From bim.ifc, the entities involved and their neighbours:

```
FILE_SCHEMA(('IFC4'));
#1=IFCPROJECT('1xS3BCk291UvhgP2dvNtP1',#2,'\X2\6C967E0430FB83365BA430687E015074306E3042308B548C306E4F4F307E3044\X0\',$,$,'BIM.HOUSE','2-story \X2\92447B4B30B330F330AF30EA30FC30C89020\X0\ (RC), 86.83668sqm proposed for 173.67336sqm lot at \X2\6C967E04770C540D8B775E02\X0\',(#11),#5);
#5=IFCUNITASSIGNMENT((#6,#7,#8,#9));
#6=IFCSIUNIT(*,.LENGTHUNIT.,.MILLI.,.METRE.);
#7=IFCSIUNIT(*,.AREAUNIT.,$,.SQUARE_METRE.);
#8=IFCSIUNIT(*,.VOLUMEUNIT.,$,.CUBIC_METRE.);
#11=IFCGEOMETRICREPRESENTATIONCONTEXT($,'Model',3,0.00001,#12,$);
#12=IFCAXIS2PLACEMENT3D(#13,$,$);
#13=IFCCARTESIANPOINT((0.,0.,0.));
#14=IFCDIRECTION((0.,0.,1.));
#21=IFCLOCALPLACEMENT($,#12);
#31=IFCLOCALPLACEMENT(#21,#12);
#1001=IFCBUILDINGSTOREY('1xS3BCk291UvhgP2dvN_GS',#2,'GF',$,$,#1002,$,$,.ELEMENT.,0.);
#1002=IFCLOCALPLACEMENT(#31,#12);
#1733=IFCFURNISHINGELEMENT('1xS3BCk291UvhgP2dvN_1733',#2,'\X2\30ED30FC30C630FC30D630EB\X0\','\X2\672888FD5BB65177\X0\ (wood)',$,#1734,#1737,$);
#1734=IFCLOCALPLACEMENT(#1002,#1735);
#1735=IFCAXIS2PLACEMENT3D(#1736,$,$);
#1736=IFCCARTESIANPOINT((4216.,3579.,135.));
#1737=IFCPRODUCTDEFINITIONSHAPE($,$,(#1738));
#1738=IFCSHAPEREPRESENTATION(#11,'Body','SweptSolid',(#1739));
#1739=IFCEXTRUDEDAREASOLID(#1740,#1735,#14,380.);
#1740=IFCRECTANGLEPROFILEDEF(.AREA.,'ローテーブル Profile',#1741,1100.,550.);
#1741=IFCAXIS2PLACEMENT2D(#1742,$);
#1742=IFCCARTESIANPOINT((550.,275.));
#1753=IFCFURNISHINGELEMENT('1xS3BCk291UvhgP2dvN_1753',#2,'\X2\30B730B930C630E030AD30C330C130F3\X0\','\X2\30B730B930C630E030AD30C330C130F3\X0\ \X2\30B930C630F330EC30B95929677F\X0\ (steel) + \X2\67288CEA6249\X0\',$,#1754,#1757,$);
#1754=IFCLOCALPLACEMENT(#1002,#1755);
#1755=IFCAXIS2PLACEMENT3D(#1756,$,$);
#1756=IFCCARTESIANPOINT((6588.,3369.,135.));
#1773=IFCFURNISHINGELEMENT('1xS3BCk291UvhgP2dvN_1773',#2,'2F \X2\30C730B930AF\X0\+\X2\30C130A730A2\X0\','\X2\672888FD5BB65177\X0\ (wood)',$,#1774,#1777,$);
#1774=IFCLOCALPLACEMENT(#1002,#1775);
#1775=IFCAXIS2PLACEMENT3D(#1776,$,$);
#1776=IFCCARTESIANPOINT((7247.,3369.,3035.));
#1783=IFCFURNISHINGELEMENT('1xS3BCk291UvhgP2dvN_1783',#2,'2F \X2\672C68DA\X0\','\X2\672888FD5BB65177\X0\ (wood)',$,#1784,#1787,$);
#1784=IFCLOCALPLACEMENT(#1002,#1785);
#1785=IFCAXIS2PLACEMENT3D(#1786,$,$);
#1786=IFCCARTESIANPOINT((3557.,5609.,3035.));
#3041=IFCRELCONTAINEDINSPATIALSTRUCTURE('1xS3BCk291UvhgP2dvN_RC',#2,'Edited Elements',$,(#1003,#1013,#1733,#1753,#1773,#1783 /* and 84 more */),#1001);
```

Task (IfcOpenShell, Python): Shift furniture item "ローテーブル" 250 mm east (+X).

```python
import ifcopenshell
import ifcopenshell.api.geometry
import ifcopenshell.util.placement
import ifcopenshell.util.unit

model = ifcopenshell.open("bim.ifc")
unit_scale = ifcopenshell.util.unit.calculate_unit_scale(model)

item = model.by_guid("1xS3BCk291UvhgP2dvN_1733")
matrix = ifcopenshell.util.placement.get_local_placement(item.ObjectPlacement)
matrix[0, 3] += 0.25 / unit_scale
ifcopenshell.api.geometry.edit_object_placement(model, product=item, matrix=matrix, is_si=False)

print(ifcopenshell.util.placement.get_local_placement(item.ObjectPlacement).round(3) + 0.0)

model.write("bim_edited.ifc")
```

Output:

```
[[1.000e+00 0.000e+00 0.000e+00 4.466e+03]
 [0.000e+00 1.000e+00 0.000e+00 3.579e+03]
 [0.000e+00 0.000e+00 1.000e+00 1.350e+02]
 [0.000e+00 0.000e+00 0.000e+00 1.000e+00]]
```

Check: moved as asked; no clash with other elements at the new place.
